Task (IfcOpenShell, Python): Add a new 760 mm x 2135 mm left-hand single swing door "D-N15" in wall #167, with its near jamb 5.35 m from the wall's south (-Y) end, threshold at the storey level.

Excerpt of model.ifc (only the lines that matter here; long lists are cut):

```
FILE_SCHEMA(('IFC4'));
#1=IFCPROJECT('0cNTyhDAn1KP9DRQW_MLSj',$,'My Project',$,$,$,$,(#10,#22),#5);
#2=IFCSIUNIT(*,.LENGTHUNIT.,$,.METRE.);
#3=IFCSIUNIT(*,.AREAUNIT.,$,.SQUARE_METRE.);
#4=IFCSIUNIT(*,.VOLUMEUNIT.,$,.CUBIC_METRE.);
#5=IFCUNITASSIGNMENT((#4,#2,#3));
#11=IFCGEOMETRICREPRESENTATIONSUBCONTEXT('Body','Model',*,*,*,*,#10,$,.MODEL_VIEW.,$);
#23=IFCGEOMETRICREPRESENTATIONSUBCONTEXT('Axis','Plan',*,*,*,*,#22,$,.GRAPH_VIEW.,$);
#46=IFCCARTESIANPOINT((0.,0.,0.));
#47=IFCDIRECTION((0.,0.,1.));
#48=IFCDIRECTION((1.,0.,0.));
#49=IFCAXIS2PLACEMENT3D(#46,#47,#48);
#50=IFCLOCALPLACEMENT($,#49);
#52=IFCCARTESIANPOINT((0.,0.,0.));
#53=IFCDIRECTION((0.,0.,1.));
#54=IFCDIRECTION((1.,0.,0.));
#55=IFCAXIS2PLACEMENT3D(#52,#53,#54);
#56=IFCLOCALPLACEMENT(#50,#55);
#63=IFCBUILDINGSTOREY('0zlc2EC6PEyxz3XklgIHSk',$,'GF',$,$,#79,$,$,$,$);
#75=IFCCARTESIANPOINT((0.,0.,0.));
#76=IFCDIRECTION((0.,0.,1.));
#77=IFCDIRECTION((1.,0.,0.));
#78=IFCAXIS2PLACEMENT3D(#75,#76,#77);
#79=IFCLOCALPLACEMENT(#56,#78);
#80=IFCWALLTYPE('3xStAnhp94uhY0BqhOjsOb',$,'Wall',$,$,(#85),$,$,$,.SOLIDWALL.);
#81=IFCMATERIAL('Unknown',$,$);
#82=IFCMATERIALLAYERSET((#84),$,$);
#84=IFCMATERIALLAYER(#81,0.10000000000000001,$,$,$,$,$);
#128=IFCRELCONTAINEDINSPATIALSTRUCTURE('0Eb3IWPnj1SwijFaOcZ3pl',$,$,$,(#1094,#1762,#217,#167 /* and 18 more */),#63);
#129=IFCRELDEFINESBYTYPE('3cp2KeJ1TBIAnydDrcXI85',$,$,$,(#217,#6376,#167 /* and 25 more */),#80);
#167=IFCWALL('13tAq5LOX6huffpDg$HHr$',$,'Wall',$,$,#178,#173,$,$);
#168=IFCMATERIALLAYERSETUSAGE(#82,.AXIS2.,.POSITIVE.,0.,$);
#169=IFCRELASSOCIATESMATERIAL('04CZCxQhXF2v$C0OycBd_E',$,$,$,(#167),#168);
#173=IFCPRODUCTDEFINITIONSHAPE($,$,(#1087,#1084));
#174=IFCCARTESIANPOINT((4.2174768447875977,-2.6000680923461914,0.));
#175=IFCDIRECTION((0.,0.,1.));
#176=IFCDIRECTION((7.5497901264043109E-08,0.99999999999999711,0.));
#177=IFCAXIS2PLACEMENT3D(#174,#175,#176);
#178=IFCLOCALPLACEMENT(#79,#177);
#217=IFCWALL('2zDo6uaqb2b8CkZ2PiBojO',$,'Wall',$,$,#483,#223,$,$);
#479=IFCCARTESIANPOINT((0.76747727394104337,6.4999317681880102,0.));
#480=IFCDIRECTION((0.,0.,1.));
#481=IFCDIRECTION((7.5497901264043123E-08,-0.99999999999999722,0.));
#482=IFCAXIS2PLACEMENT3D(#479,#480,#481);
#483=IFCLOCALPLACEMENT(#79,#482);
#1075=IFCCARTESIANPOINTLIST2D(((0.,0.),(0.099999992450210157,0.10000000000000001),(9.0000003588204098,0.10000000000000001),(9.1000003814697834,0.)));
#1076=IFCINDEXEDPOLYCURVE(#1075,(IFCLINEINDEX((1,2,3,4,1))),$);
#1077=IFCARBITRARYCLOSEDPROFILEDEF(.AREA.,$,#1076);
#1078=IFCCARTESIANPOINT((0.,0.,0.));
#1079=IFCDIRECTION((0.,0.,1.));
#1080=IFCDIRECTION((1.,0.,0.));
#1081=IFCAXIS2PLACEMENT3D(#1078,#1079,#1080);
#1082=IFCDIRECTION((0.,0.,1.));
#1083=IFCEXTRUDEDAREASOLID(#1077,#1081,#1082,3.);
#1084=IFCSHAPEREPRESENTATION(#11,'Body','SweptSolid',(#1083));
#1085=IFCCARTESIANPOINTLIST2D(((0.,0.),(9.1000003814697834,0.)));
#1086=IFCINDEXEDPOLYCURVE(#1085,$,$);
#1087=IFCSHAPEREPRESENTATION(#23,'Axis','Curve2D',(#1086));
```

```python
import numpy as np
import ifcopenshell
import ifcopenshell.api.feature
import ifcopenshell.api.geometry
import ifcopenshell.api.root
import ifcopenshell.api.spatial
import ifcopenshell.geom
import ifcopenshell.util.element
import ifcopenshell.util.placement
import ifcopenshell.util.representation
import ifcopenshell.util.shape
import ifcopenshell.util.unit

model = ifcopenshell.open("model.ifc")
unit_scale = ifcopenshell.util.unit.calculate_unit_scale(model)
settings = ifcopenshell.geom.settings()


def volume(element):
    """Net volume in cubic metres, openings subtracted."""
    shape = ifcopenshell.geom.create_shape(settings, element)
    return ifcopenshell.util.shape.get_volume(shape.geometry)


wall = model.by_guid("13tAq5LOX6huffpDg$HHr$")
storey = ifcopenshell.util.element.get_container(wall, ifc_class="IfcBuildingStorey")
context = ifcopenshell.util.representation.get_context(model, "Model", "Body", "MODEL_VIEW")
before = volume(wall)

width, height, from_end, sill = 0.76, 2.135, 5.35, 0.0  # metres

# The wall runs along its own X axis, and the end named is its -X end.
wall_shape = ifcopenshell.geom.create_shape(settings, wall)
x, y, z = ifcopenshell.util.shape.get_vertices(wall_shape.geometry).T
start = x.min() + from_end
face, thickness = float(y.min()), float(y.max() - y.min())
wall_matrix = ifcopenshell.util.placement.get_local_placement(wall.ObjectPlacement)
level = ifcopenshell.util.placement.get_local_placement(storey.ObjectPlacement)[2, 3]


def in_wall(x, y):
    """Placement at x, y metres in the wall's axes, at sill height."""
    matrix = wall_matrix.copy()
    matrix[:, 3] = wall_matrix @ np.array([x / unit_scale, y / unit_scale, 0.0, 1.0])
    matrix[2, 3] = level + sill / unit_scale
    return matrix


# Opening: a box that overshoots both wall faces by 50 mm.
opening = ifcopenshell.api.root.create_entity(model, ifc_class="IfcOpeningElement", predefined_type="OPENING")
box = ifcopenshell.api.geometry.add_wall_representation(
    model, context=context, length=width, height=height, thickness=thickness + 0.1
)
ifcopenshell.api.geometry.assign_representation(model, product=opening, representation=box)
ifcopenshell.api.geometry.edit_object_placement(model, product=opening, matrix=in_wall(start, face - 0.05), is_si=False)
ifcopenshell.api.feature.add_feature(model, feature=opening, element=wall)

door = ifcopenshell.api.root.create_entity(model, ifc_class="IfcDoor", name="D-N15", predefined_type="DOOR")
door.OverallWidth, door.OverallHeight = width / unit_scale, height / unit_scale
door.OperationType = "SINGLE_SWING_LEFT"
body = ifcopenshell.api.geometry.add_door_representation(
    model,
    context=context,
    overall_width=door.OverallWidth,
    overall_height=door.OverallHeight,
    operation_type="SINGLE_SWING_LEFT",
    lining_properties={"LiningDepth": thickness / unit_scale, "ThresholdDepth": thickness / unit_scale},
)
ifcopenshell.api.geometry.assign_representation(model, product=door, representation=body)
ifcopenshell.api.spatial.assign_container(model, products=[door], relating_structure=storey)
ifcopenshell.api.feature.add_filling(model, opening=opening, element=door)

# The lining spans the wall, so the door starts at the wall face.
ifcopenshell.api.geometry.edit_object_placement(model, product=door, matrix=in_wall(start, face), is_si=False)

after = volume(wall)

print(f"wall volume {before:.3f} -> {after:.3f} m3")

model.write("model_v2.ifc")
```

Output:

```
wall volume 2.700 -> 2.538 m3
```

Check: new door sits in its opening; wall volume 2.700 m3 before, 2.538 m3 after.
